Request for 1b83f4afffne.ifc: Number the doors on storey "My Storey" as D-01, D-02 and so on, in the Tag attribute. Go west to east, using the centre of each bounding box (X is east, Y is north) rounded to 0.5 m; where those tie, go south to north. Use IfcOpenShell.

First a look at what the model holds.

```python
import ifcopenshell
import ifcopenshell.util.element
import ifcopenshell.util.placement

model = ifcopenshell.open("1b83f4afffne.ifc")
print(model.schema)
storey = next(s for s in model.by_type("IfcBuildingStorey") if s.Name == "My Storey")
doors = [e for e in ifcopenshell.util.element.get_decomposition(storey) if e.is_a("IfcDoor")]
for e in sorted(doors, key=lambda e: e.id()):
    origin = ifcopenshell.util.placement.get_local_placement(e.ObjectPlacement)[:3, 3]
    print(e.id(), e.Tag, e.Name, origin.round(2) + 0.0, sep=" | ")
```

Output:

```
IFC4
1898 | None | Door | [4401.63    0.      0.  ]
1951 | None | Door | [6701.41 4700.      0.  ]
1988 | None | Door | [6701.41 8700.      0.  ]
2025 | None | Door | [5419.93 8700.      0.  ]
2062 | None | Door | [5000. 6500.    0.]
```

```python
import ifcopenshell
import ifcopenshell.geom
import ifcopenshell.util.element
import ifcopenshell.util.shape

model = ifcopenshell.open("1b83f4afffne.ifc")
settings = ifcopenshell.geom.settings()
settings.set("use-world-coords", True)


def centre(element):
    shape = ifcopenshell.geom.create_shape(settings, element)
    return ifcopenshell.util.shape.get_bbox_centroid(shape.geometry)


storey = next(s for s in model.by_type("IfcBuildingStorey") if s.Name == "My Storey")
doors = [e for e in ifcopenshell.util.element.get_decomposition(storey) if e.is_a("IfcDoor")]

# Insertion points can sit at a corner or the storey origin, so sort by the geometry (in metres).
centres = {e: centre(e) for e in doors}
doors.sort(key=lambda e: (round(centres[e][0] / 0.5), centres[e][1]))

for i, e in enumerate(doors, start=1):
    number = f"D-{i:02d}"
    e.Tag = number
    print(e.id(), number)

model.write("1b83f4afffne_edited.ifc")
```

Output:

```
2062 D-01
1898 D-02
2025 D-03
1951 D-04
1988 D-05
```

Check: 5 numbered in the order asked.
